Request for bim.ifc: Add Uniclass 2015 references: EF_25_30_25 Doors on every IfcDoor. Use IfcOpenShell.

First a look at what the model holds.

```python
import ifcopenshell

model = ifcopenshell.open("bim.ifc")
print(model.schema)
print("classifications:", [c.Name for c in model.by_type("IfcClassification")])
for ifc_class in ("IfcDoor", "IfcRoof", "IfcStair", "IfcWall", "IfcWindow"):
    print(ifc_class, len(model.by_type(ifc_class)))
```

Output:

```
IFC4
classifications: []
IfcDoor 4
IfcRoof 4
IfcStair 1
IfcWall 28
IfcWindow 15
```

```python
import ifcopenshell
import ifcopenshell.api.classification

model = ifcopenshell.open("bim.ifc")

system = ifcopenshell.api.classification.add_classification(model, classification="Uniclass 2015")

codes = {
    "IfcDoor": ("EF_25_30_25", "Doors"),
}
for ifc_class, (code, name) in codes.items():
    products = model.by_type(ifc_class)
    ifcopenshell.api.classification.add_reference(
        model, products=products, classification=system, identification=code, name=name
    )
    print(code, len(products))

model.write("bim_v2.ifc")
```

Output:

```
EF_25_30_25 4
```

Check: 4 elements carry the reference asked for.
